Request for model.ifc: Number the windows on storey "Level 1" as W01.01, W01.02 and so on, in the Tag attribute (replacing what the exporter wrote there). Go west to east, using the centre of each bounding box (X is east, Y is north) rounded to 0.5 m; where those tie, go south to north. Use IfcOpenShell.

First a look at what the model holds.

```python
import ifcopenshell
import ifcopenshell.util.element
import ifcopenshell.util.placement

model = ifcopenshell.open("model.ifc")
print(model.schema)
storey = next(s for s in model.by_type("IfcBuildingStorey") if s.Name == "Level 1")
windows = [e for e in ifcopenshell.util.element.get_decomposition(storey) if e.is_a("IfcWindow")]
for e in sorted(windows, key=lambda e: e.id()):
    origin = ifcopenshell.util.placement.get_local_placement(e.ObjectPlacement)[:3, 3]
    print(e.id(), e.Tag, e.Name, origin.round(2) + 0.0, sep=" | ")
```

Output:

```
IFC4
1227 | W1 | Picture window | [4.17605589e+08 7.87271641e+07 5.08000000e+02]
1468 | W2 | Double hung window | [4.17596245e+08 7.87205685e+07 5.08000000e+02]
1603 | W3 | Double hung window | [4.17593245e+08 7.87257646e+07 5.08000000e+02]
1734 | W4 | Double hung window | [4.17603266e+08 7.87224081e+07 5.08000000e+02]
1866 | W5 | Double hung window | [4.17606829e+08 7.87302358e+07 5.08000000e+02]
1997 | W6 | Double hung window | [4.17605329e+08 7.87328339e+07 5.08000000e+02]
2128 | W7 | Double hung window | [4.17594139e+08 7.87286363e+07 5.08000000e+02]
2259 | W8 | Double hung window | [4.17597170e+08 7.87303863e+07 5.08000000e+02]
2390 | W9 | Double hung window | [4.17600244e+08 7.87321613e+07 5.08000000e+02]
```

```python
import ifcopenshell
import ifcopenshell.geom
import ifcopenshell.util.element
import ifcopenshell.util.shape

model = ifcopenshell.open("model.ifc")
settings = ifcopenshell.geom.settings()
settings.set("use-world-coords", True)


def centre(element):
    shape = ifcopenshell.geom.create_shape(settings, element)
    return ifcopenshell.util.shape.get_bbox_centroid(shape.geometry)


storey = next(s for s in model.by_type("IfcBuildingStorey") if s.Name == "Level 1")
windows = [e for e in ifcopenshell.util.element.get_decomposition(storey) if e.is_a("IfcWindow")]

# Insertion points can sit at a corner or the storey origin, so sort by the geometry (in metres).
centres = {e: centre(e) for e in windows}
windows.sort(key=lambda e: (round(centres[e][0] / 0.5), centres[e][1]))

for i, e in enumerate(windows, start=1):
    number = f"W01.{i:02d}"
    e.Tag = number
    print(e.id(), number)

model.write("model_updated.ifc")
```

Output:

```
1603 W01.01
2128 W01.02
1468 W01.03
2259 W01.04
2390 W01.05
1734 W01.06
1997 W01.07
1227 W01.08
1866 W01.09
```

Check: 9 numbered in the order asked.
